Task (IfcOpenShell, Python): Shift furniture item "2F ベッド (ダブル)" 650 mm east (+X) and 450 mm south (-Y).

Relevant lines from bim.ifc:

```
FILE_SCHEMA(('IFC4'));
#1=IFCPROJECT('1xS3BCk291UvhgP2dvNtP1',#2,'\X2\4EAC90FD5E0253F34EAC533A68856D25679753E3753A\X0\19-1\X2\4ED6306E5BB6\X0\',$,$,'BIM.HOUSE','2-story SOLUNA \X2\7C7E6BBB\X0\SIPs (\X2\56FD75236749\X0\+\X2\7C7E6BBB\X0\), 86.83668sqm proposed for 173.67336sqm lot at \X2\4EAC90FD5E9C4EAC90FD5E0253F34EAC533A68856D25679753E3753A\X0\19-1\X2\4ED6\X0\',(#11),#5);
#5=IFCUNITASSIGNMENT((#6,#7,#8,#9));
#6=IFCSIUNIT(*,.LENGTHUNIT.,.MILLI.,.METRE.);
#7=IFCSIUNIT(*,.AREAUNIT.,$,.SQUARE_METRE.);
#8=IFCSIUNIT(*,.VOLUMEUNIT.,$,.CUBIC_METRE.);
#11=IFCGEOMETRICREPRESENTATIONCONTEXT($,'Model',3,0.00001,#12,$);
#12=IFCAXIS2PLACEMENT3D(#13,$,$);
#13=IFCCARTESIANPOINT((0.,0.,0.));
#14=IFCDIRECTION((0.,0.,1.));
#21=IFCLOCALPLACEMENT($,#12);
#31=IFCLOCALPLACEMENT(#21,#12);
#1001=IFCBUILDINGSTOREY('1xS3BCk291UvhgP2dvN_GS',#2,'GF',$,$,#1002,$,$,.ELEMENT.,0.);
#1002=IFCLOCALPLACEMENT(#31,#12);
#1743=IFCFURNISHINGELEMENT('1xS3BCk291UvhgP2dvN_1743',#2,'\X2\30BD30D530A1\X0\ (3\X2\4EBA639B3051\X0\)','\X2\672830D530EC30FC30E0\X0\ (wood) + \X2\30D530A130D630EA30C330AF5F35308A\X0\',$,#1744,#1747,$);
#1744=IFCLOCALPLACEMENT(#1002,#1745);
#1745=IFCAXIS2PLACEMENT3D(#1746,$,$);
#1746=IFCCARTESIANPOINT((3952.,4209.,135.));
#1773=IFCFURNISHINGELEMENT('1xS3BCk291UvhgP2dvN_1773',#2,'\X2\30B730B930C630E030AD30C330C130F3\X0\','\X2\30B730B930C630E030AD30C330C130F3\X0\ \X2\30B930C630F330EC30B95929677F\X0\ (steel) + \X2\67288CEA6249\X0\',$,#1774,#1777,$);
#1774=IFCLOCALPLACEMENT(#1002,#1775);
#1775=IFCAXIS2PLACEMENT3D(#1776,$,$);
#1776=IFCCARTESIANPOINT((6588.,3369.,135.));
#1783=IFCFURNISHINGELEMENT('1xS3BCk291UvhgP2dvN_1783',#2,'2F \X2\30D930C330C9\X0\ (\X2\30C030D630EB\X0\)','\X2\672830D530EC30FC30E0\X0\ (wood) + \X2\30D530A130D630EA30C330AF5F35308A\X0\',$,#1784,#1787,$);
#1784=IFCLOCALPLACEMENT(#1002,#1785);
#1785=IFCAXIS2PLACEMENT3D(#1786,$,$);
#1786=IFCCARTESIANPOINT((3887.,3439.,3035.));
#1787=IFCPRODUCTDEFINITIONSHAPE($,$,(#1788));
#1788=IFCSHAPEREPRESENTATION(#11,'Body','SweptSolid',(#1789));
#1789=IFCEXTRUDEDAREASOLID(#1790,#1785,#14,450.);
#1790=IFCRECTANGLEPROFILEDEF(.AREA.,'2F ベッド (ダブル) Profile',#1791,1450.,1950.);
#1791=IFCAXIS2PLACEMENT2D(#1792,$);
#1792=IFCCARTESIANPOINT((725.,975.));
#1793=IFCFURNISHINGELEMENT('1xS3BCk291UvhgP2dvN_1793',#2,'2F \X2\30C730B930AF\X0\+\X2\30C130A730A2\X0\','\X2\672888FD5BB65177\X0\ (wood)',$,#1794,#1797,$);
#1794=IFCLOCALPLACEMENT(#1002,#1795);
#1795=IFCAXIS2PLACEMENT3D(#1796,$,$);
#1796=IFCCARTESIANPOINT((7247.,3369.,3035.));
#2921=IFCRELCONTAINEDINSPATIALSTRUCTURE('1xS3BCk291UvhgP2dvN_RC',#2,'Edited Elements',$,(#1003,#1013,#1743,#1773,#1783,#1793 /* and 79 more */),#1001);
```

```python
import ifcopenshell
import ifcopenshell.api.geometry
import ifcopenshell.util.placement
import ifcopenshell.util.unit

model = ifcopenshell.open("bim.ifc")
unit_scale = ifcopenshell.util.unit.calculate_unit_scale(model)

item = model.by_guid("1xS3BCk291UvhgP2dvN_1783")
matrix = ifcopenshell.util.placement.get_local_placement(item.ObjectPlacement)
matrix[0, 3] += 0.65 / unit_scale
matrix[1, 3] -= 0.45 / unit_scale
ifcopenshell.api.geometry.edit_object_placement(model, product=item, matrix=matrix, is_si=False)

print(ifcopenshell.util.placement.get_local_placement(item.ObjectPlacement).round(3) + 0.0)

model.write("bim-out.ifc")
```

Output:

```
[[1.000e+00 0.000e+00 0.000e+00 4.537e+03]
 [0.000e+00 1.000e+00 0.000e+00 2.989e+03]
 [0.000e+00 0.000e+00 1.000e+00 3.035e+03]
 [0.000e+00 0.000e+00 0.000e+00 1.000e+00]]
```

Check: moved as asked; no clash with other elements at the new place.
